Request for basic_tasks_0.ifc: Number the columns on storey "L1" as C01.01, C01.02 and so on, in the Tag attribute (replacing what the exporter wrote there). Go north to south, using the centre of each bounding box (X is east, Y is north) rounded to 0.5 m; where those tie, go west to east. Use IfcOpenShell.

First a look at what the model holds.

```python
import ifcopenshell
import ifcopenshell.util.element
import ifcopenshell.util.placement

model = ifcopenshell.open("basic_tasks_0.ifc")
print(model.schema)
storey = next(s for s in model.by_type("IfcBuildingStorey") if s.Name == "L1")
columns = [e for e in ifcopenshell.util.element.get_decomposition(storey) if e.is_a("IfcColumn")]
for e in sorted(columns, key=lambda e: e.id()):
    origin = ifcopenshell.util.placement.get_local_placement(e.ObjectPlacement)[:3, 3]
    print(e.id(), e.Tag, e.Name, origin.round(2) + 0.0, sep=" | ")
```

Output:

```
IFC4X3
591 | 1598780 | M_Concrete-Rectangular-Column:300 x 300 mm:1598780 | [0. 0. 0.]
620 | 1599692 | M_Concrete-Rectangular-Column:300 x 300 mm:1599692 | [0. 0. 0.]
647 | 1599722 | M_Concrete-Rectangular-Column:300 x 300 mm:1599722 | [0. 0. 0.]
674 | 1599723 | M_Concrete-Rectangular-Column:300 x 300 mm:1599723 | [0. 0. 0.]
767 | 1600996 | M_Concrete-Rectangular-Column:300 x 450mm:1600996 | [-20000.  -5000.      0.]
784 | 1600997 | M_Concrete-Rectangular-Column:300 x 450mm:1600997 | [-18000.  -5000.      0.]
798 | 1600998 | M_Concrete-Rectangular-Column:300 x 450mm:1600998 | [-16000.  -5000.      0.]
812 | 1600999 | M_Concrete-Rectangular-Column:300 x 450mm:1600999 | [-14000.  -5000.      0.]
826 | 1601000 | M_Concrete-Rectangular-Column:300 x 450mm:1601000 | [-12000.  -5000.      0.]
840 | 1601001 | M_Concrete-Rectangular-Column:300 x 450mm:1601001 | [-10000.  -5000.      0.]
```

```python
import ifcopenshell
import ifcopenshell.geom
import ifcopenshell.util.element
import ifcopenshell.util.shape

model = ifcopenshell.open("basic_tasks_0.ifc")
settings = ifcopenshell.geom.settings()
settings.set("use-world-coords", True)


def centre(element):
    shape = ifcopenshell.geom.create_shape(settings, element)
    return ifcopenshell.util.shape.get_bbox_centroid(shape.geometry)


storey = next(s for s in model.by_type("IfcBuildingStorey") if s.Name == "L1")
columns = [e for e in ifcopenshell.util.element.get_decomposition(storey) if e.is_a("IfcColumn")]

# Insertion points can sit at a corner or the storey origin, so sort by the geometry (in metres).
centres = {e: centre(e) for e in columns}
columns.sort(key=lambda e: (-round(centres[e][1] / 0.5), centres[e][0]))

for i, e in enumerate(columns, start=1):
    number = f"C01.{i:02d}"
    e.Tag = number
    print(e.id(), number)

model.write("basic_tasks_0_v2.ifc")
```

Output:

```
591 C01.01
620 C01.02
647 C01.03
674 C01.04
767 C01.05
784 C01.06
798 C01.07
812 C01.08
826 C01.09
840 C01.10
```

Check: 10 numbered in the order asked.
